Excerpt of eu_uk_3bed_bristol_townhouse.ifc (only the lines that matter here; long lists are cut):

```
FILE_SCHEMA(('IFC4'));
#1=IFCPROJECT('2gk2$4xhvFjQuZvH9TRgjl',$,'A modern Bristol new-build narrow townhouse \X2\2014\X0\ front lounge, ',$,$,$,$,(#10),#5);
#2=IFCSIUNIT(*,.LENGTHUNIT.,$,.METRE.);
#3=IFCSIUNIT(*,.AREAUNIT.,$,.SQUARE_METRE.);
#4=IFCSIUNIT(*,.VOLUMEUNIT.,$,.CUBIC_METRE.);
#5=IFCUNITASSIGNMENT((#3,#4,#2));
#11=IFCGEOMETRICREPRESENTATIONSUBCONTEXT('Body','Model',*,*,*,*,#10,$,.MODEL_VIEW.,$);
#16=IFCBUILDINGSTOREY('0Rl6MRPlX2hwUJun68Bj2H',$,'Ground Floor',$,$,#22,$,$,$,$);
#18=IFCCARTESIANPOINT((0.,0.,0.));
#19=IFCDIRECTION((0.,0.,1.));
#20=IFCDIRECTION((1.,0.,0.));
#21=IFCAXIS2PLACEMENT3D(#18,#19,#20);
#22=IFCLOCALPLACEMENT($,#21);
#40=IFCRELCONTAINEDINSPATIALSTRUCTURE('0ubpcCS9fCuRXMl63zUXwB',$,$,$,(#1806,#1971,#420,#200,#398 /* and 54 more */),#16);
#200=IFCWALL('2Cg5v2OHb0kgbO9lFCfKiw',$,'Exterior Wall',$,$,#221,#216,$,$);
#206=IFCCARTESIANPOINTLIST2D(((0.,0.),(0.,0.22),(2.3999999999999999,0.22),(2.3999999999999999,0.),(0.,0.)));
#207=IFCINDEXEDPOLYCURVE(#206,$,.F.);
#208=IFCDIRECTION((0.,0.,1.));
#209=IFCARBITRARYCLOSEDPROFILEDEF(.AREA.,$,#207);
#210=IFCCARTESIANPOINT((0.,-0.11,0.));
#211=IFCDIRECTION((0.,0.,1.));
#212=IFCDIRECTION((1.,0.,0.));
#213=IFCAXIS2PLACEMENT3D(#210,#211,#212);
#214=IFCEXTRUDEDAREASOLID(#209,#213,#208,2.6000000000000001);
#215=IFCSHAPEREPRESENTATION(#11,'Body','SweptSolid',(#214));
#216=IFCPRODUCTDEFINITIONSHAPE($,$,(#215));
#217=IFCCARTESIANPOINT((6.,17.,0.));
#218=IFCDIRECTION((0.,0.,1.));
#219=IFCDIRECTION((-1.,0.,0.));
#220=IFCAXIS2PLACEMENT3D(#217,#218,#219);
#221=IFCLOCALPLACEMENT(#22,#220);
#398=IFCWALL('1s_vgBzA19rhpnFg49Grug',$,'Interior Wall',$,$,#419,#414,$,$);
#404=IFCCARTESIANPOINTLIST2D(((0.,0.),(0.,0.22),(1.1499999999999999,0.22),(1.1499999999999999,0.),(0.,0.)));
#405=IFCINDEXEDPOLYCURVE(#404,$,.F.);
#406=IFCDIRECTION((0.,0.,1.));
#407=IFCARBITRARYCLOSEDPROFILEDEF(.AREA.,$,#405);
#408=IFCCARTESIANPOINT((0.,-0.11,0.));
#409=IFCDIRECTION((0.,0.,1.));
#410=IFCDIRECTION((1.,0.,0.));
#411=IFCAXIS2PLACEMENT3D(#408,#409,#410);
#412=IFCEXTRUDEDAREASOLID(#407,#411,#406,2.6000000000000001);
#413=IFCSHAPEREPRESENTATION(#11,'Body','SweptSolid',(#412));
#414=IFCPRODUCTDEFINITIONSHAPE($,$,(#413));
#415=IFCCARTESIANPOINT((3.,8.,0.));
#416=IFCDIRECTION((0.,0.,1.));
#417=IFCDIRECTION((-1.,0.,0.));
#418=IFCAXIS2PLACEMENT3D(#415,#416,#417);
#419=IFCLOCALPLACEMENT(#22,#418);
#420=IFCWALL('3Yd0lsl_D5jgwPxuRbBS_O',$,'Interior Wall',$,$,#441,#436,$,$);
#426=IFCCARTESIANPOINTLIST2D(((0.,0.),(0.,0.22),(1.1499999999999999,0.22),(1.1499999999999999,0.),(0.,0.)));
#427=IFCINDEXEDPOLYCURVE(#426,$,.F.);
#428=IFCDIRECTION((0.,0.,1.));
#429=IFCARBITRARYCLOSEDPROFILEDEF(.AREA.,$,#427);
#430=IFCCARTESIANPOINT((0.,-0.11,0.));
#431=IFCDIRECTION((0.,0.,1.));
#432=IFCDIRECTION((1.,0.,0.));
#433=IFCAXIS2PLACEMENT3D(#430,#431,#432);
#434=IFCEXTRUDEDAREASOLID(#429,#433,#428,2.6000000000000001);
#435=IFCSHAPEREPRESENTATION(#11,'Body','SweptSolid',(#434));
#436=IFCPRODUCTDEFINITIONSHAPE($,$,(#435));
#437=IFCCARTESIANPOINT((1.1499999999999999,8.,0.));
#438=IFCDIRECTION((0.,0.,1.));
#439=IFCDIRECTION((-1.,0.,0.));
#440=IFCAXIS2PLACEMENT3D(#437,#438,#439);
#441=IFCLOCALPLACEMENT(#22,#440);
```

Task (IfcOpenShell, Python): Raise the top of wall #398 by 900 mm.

```python
import ifcopenshell
import ifcopenshell.geom
import ifcopenshell.util.representation
import ifcopenshell.util.shape
import ifcopenshell.util.unit

model = ifcopenshell.open("eu_uk_3bed_bristol_townhouse.ifc")
unit_scale = ifcopenshell.util.unit.calculate_unit_scale(model)
settings = ifcopenshell.geom.settings()


def volume(element):
    """Net volume in cubic metres, openings subtracted."""
    shape = ifcopenshell.geom.create_shape(settings, element)
    return ifcopenshell.util.shape.get_volume(shape.geometry)


wall = model.by_id(398)
before = volume(wall)

body = ifcopenshell.util.representation.get_representation(wall, "Model", "Body")
solid = body.Items[0]
old_height = solid.Depth
solid.Depth += 0.9 / unit_scale
after = volume(wall)

print(f"height {old_height:g} -> {solid.Depth:g}, volume {before:.3f} -> {after:.3f} m3")

model.write("eu_uk_3bed_bristol_townhouse-out.ifc")
```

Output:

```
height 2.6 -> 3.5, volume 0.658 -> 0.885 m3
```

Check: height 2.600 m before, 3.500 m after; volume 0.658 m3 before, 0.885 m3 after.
